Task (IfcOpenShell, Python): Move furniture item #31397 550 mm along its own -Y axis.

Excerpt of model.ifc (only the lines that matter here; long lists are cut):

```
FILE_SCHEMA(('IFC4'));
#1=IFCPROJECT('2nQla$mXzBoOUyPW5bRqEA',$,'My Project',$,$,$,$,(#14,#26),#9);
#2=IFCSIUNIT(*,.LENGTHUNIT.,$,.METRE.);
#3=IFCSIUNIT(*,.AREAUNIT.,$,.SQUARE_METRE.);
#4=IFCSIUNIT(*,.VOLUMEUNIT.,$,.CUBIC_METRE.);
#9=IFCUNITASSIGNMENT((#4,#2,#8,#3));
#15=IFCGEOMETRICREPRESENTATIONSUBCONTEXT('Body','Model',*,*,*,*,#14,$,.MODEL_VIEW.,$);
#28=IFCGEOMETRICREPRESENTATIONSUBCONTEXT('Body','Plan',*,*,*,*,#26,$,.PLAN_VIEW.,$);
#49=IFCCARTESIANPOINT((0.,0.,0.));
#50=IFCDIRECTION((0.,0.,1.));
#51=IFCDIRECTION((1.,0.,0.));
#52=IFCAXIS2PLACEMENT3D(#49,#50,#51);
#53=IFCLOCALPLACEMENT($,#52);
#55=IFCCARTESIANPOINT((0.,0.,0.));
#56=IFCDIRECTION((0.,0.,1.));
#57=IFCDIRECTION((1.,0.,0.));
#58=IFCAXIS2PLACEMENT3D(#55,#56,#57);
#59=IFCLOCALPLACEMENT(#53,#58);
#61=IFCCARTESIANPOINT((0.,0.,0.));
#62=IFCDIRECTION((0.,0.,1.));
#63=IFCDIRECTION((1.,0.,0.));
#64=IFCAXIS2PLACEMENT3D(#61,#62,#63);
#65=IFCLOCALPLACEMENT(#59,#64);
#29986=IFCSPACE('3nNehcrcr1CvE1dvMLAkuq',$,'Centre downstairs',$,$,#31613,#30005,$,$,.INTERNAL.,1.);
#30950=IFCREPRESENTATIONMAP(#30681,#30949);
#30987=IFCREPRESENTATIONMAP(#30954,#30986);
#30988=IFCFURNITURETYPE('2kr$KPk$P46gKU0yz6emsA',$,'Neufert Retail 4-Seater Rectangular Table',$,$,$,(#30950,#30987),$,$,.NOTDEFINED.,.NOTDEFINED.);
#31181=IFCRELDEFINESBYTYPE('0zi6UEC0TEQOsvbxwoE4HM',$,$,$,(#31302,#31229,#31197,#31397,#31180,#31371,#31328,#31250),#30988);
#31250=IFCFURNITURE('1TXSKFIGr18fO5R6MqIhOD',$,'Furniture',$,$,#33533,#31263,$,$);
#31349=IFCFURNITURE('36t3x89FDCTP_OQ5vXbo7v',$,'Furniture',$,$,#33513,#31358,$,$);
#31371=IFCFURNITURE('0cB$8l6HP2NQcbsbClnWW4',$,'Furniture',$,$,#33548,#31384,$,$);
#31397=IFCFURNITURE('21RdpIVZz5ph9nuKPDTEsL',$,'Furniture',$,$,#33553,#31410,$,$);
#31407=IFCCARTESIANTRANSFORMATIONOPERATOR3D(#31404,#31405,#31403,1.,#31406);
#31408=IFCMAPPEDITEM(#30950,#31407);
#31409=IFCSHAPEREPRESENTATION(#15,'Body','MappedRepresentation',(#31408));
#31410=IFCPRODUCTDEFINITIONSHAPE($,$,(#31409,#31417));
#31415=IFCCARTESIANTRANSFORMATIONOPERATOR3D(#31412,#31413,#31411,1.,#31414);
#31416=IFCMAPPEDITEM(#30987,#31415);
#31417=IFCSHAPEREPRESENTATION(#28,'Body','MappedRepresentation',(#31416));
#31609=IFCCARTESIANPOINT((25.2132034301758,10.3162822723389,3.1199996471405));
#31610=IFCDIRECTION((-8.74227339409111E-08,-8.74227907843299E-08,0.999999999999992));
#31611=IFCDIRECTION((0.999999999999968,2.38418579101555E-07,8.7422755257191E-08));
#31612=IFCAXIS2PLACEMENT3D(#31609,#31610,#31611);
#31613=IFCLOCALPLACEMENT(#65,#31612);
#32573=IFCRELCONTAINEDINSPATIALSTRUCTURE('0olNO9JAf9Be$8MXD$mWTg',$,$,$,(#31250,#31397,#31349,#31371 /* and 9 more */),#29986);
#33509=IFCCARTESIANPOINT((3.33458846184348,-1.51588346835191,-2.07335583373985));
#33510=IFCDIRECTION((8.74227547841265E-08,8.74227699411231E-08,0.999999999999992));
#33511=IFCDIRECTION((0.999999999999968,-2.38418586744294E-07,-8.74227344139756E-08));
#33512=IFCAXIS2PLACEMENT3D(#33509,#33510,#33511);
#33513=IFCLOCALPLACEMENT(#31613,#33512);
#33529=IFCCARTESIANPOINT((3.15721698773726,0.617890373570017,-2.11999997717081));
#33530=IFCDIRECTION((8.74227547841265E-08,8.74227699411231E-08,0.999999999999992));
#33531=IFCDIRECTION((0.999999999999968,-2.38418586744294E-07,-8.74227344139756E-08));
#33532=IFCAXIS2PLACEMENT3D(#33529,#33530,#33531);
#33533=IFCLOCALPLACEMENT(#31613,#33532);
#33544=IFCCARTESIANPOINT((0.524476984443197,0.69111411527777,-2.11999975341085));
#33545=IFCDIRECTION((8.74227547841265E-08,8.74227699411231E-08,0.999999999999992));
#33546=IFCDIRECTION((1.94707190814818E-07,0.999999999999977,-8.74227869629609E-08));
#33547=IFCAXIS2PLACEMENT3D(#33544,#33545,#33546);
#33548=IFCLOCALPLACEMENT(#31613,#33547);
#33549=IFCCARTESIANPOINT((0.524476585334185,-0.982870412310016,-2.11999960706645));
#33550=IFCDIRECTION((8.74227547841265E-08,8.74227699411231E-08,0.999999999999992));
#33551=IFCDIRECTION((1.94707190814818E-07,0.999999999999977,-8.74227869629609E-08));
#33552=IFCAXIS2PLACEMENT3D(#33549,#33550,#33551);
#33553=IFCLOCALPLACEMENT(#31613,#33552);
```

```python
import ifcopenshell
import ifcopenshell.api.geometry
import ifcopenshell.util.placement
import ifcopenshell.util.unit

model = ifcopenshell.open("model.ifc")
unit_scale = ifcopenshell.util.unit.calculate_unit_scale(model)

item = model.by_id(31397)
matrix = ifcopenshell.util.placement.get_local_placement(item.ObjectPlacement)
matrix[:3, 3] -= matrix[:3, 1] * 0.55 / unit_scale
ifcopenshell.api.geometry.edit_object_placement(model, product=item, matrix=matrix, is_si=False)

print(ifcopenshell.util.placement.get_local_placement(item.ObjectPlacement).round(3) + 0.0)

model.write("model_rev.ifc")
```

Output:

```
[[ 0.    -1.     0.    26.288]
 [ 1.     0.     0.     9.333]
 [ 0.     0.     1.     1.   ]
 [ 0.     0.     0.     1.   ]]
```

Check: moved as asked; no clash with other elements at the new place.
